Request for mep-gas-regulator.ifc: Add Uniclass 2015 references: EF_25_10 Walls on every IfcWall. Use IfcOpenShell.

First a look at what the model holds.

```python
import ifcopenshell

model = ifcopenshell.open("mep-gas-regulator.ifc")
print(model.schema)
print("classifications:", [c.Name for c in model.by_type("IfcClassification")])
for ifc_class in ("IfcDoor", "IfcRoof", "IfcStair", "IfcWall", "IfcWindow"):
    print(ifc_class, len(model.by_type(ifc_class)))
```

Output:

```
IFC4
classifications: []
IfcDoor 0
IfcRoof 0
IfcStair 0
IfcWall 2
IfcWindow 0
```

```python
import ifcopenshell
import ifcopenshell.api.classification

model = ifcopenshell.open("mep-gas-regulator.ifc")

system = ifcopenshell.api.classification.add_classification(model, classification="Uniclass 2015")

codes = {
    "IfcWall": ("EF_25_10", "Walls"),
}
for ifc_class, (code, name) in codes.items():
    products = model.by_type(ifc_class)
    ifcopenshell.api.classification.add_reference(
        model, products=products, classification=system, identification=code, name=name
    )
    print(code, len(products))

model.write("mep-gas-regulator_updated.ifc")
```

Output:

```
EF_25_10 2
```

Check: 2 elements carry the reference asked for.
